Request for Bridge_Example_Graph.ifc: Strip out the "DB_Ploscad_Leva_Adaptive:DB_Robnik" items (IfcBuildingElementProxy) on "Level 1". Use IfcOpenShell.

First a look at what the model holds.

```python
import ifcopenshell
import ifcopenshell.util.element

model = ifcopenshell.open("Bridge_Example_Graph.ifc")
print(model.schema)
storey = next(s for s in model.by_type("IfcBuildingStorey") if s.Name == "Level 1")
proxies = [e for e in ifcopenshell.util.element.get_decomposition(storey) if e.is_a("IfcBuildingElementProxy")]
seen = {}
for e in proxies:
    element_type = ifcopenshell.util.element.get_type(e)
    name = element_type.Name if element_type not in (None, e) else None
    seen[name] = seen.get(name, 0) + 1
for name, count in sorted(seen.items(), key=str):
    print(count, "x", name)
```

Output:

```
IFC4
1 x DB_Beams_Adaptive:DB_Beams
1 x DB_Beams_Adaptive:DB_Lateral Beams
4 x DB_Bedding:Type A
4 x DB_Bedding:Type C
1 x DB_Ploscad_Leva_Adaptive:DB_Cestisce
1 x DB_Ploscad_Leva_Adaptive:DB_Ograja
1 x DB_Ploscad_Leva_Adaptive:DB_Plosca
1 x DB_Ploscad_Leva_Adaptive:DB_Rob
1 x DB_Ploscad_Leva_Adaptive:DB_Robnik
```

```python
import ifcopenshell
import ifcopenshell.api.root
import ifcopenshell.util.element

model = ifcopenshell.open("Bridge_Example_Graph.ifc")

storey = next(s for s in model.by_type("IfcBuildingStorey") if s.Name == "Level 1")
proxies = [e for e in ifcopenshell.util.element.get_decomposition(storey) if e.is_a("IfcBuildingElementProxy")]
targets = [e for e in proxies if (t := ifcopenshell.util.element.get_type(e)) not in (None, e) and t.Name == "DB_Ploscad_Leva_Adaptive:DB_Robnik"]

for e in targets:
    ifcopenshell.api.root.remove_product(model, product=e)
print(len(targets), "removed")

model.write("Bridge_Example_Graph-out.ifc")
```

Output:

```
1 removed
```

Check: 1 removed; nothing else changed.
